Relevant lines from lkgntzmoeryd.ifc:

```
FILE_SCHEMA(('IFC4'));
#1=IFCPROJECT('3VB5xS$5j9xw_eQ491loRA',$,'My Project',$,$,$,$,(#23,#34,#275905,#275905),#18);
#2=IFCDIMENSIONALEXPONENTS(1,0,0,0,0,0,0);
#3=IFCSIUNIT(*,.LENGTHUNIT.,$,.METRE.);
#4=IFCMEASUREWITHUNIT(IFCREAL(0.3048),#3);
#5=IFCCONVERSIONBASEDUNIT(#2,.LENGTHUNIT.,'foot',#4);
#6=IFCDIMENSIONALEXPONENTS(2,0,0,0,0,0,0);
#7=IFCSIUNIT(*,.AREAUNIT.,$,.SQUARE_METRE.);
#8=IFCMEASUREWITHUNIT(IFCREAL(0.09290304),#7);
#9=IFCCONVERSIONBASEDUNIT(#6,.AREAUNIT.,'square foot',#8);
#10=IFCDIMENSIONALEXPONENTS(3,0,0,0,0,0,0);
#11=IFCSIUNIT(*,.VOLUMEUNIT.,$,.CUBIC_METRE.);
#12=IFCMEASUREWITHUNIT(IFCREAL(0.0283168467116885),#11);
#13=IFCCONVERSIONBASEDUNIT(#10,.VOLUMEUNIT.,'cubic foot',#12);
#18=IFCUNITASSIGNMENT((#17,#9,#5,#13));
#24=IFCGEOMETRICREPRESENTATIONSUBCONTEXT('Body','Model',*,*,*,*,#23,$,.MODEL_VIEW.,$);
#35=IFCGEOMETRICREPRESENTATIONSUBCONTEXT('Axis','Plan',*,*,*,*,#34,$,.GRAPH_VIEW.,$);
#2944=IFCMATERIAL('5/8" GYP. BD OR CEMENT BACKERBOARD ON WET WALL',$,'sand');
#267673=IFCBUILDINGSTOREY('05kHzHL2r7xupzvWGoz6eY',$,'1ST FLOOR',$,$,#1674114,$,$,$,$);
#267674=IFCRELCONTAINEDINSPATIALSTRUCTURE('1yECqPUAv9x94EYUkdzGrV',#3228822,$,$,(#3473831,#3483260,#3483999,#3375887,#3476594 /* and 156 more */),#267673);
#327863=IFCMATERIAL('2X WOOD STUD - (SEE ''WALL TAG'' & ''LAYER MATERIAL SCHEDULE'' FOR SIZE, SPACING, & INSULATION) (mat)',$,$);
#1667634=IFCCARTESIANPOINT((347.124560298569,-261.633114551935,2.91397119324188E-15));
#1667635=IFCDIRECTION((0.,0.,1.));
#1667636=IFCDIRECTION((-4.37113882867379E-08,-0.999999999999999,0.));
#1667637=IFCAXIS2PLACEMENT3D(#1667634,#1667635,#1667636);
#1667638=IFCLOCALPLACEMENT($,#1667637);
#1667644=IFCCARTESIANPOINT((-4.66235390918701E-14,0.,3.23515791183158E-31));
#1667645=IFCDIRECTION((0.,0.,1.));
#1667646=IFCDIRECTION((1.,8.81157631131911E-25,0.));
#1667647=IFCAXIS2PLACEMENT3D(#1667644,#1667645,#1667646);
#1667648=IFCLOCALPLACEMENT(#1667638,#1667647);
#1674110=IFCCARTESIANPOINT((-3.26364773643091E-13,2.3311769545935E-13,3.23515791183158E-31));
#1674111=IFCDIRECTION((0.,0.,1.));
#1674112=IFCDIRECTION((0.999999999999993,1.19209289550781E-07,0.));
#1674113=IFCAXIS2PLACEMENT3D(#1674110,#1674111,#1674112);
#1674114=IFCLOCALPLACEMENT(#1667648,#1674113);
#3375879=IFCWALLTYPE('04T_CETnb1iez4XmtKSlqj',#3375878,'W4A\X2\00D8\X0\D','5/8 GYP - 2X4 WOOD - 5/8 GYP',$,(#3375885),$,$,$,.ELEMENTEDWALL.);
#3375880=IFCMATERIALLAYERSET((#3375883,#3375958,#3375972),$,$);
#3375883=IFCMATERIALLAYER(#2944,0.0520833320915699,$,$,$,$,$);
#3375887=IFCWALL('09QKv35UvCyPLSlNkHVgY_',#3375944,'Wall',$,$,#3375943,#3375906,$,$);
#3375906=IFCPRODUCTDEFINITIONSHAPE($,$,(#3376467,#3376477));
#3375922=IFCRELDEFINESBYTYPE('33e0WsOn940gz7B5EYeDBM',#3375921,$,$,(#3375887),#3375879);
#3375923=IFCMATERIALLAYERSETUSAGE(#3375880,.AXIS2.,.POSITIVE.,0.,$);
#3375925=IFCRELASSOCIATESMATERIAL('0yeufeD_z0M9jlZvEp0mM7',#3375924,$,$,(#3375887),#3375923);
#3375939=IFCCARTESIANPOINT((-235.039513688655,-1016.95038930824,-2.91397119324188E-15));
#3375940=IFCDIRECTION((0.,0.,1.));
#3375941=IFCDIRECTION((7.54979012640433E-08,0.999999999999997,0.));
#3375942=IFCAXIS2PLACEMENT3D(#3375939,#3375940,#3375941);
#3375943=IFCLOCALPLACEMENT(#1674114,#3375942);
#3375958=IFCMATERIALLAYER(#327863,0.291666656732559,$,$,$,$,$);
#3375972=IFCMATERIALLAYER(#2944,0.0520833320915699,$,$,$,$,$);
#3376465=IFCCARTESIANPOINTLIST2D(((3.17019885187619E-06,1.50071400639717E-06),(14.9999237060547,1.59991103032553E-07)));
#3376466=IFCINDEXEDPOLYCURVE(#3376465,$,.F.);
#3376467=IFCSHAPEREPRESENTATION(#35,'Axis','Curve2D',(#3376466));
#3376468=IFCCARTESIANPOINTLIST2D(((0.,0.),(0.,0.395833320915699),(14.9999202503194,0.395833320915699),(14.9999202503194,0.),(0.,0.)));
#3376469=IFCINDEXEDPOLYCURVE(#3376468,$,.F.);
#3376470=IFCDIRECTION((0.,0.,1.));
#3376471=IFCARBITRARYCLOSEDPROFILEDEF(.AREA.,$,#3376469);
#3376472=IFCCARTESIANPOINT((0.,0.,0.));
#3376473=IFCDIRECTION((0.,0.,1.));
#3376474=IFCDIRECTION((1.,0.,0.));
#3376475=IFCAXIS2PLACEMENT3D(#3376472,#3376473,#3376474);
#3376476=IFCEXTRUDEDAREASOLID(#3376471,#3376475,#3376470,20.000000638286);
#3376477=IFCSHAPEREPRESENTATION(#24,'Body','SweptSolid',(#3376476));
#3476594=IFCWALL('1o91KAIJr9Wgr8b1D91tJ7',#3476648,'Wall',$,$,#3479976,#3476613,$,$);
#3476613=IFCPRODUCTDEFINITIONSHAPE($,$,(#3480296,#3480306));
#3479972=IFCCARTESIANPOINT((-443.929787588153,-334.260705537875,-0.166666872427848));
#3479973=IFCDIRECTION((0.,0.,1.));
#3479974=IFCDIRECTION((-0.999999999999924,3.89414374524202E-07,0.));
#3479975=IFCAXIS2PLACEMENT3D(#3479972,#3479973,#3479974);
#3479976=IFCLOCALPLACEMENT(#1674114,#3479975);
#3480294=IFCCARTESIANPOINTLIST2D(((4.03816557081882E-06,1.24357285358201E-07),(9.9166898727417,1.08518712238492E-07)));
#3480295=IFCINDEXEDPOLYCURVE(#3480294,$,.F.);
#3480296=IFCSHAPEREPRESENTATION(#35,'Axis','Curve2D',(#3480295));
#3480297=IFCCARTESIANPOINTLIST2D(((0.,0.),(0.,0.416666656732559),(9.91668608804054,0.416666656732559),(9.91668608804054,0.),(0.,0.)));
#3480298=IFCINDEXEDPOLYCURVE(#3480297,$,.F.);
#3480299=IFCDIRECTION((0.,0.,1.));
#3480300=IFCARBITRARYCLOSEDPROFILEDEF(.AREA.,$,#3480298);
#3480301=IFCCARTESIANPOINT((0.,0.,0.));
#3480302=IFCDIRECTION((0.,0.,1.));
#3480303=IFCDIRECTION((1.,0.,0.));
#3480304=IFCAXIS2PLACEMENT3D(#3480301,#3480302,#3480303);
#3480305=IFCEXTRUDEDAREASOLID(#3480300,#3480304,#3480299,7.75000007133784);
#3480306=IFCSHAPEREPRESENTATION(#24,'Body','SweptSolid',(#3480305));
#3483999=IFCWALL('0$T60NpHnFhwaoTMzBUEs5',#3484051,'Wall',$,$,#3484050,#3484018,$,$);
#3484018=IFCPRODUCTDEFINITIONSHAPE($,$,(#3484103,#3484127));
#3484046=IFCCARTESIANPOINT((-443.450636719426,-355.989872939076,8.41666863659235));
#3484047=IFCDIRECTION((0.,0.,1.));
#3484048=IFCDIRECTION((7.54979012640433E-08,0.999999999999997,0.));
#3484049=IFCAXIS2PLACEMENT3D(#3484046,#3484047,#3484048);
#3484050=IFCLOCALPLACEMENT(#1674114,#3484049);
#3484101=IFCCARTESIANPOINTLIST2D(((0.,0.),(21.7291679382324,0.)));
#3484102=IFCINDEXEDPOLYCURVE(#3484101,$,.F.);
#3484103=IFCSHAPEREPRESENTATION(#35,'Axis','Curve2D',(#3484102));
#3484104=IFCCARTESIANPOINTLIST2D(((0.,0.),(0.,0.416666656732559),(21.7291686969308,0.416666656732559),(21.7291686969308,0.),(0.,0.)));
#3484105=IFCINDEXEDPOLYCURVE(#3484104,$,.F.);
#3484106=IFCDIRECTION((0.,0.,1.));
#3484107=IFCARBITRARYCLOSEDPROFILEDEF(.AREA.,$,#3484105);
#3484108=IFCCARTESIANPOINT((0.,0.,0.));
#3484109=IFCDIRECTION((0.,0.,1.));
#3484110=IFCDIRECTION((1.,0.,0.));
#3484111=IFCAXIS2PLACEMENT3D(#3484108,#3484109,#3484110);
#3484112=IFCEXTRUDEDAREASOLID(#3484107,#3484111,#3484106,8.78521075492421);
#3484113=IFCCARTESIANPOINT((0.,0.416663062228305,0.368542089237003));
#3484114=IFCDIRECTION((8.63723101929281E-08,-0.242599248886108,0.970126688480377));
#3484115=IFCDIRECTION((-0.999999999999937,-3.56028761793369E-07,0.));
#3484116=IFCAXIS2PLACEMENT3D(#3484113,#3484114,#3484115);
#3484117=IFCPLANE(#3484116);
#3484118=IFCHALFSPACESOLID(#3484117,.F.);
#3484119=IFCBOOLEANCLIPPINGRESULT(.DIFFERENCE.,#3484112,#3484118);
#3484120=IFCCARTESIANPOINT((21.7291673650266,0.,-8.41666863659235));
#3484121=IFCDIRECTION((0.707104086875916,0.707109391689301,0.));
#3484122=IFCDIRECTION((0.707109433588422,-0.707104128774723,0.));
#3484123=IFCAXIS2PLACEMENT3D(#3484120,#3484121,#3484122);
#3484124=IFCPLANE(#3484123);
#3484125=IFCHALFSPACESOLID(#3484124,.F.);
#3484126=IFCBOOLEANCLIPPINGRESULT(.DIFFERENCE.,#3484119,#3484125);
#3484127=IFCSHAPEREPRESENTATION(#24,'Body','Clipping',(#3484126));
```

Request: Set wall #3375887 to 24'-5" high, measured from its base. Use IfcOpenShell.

```python
import ifcopenshell
import ifcopenshell.geom
import ifcopenshell.util.representation
import ifcopenshell.util.shape
import ifcopenshell.util.unit

model = ifcopenshell.open("lkgntzmoeryd.ifc")
unit_scale = ifcopenshell.util.unit.calculate_unit_scale(model)
settings = ifcopenshell.geom.settings()


def volume(element):
    """Net volume in cubic metres, openings subtracted."""
    shape = ifcopenshell.geom.create_shape(settings, element)
    return ifcopenshell.util.shape.get_volume(shape.geometry)


wall = model.by_id(3375887)
before = volume(wall)

body = ifcopenshell.util.representation.get_representation(wall, "Model", "Body")
solid = body.Items[0]
old_height = solid.Depth
solid.Depth = 293 * 0.0254 / unit_scale
after = volume(wall)

print(f"height {old_height:g} -> {solid.Depth:g}, volume {before:.3f} -> {after:.3f} m3")

model.write("lkgntzmoeryd_v2.ifc")
```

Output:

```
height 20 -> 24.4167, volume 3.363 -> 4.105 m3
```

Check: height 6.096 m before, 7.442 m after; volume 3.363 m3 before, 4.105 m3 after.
